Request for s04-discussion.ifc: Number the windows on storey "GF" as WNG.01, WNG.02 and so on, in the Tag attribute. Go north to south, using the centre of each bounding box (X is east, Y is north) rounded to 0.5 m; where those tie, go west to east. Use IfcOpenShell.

First a look at what the model holds.

```python
import ifcopenshell
import ifcopenshell.util.element
import ifcopenshell.util.placement

model = ifcopenshell.open("s04-discussion.ifc")
print(model.schema)
storey = next(s for s in model.by_type("IfcBuildingStorey") if s.Name == "GF")
windows = [e for e in ifcopenshell.util.element.get_decomposition(storey) if e.is_a("IfcWindow")]
for e in sorted(windows, key=lambda e: e.id()):
    origin = ifcopenshell.util.placement.get_local_placement(e.ObjectPlacement)[:3, 3]
    print(e.id(), e.Tag, e.Name, origin.round(2) + 0.0, sep=" | ")
```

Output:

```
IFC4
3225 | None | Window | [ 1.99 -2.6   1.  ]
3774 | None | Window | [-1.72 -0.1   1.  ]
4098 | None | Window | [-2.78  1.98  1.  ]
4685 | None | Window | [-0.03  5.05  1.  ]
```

```python
import ifcopenshell
import ifcopenshell.geom
import ifcopenshell.util.element
import ifcopenshell.util.shape

model = ifcopenshell.open("s04-discussion.ifc")
settings = ifcopenshell.geom.settings()
settings.set("use-world-coords", True)


def centre(element):
    shape = ifcopenshell.geom.create_shape(settings, element)
    return ifcopenshell.util.shape.get_bbox_centroid(shape.geometry)


storey = next(s for s in model.by_type("IfcBuildingStorey") if s.Name == "GF")
windows = [e for e in ifcopenshell.util.element.get_decomposition(storey) if e.is_a("IfcWindow")]

# Insertion points can sit at a corner or the storey origin, so sort by the geometry (in metres).
centres = {e: centre(e) for e in windows}
windows.sort(key=lambda e: (-round(centres[e][1] / 0.5), centres[e][0]))

for i, e in enumerate(windows, start=1):
    number = f"WNG.{i:02d}"
    e.Tag = number
    print(e.id(), number)

model.write("s04-discussion_rev.ifc")
```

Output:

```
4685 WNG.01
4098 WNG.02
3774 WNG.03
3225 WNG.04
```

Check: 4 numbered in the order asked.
